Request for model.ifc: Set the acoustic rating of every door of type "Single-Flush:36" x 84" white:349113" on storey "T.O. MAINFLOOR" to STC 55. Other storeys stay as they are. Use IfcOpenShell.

First a look at what the model holds.

```python
import ifcopenshell
import ifcopenshell.util.element

model = ifcopenshell.open("model.ifc")
print(model.schema)
storey = next(s for s in model.by_type("IfcBuildingStorey") if s.Name == "T.O. MAINFLOOR")
doors = [e for e in ifcopenshell.util.element.get_decomposition(storey) if e.is_a("IfcDoor")]
seen = {}
for e in doors:
    element_type = ifcopenshell.util.element.get_type(e)
    key = (element_type.Name if element_type != e and element_type else None, ifcopenshell.util.element.get_pset(e, "Pset_DoorCommon", "AcousticRating"))
    seen[key] = seen.get(key, 0) + 1
for (name, value), count in sorted(seen.items(), key=str):
    print(count, "x", name, "|", value)
```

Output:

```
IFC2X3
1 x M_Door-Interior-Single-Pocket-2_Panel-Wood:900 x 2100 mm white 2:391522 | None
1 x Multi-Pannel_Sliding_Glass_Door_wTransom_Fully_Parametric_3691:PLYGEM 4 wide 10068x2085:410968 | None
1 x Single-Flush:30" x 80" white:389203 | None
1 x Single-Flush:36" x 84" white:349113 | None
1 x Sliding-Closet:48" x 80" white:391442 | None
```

```python
import ifcopenshell
import ifcopenshell.api.pset
import ifcopenshell.util.element

model = ifcopenshell.open("model.ifc")

storey = next(s for s in model.by_type("IfcBuildingStorey") if s.Name == "T.O. MAINFLOOR")
doors = [e for e in ifcopenshell.util.element.get_decomposition(storey) if e.is_a("IfcDoor")]

count = 0
for e in doors:
    element_type = ifcopenshell.util.element.get_type(e)
    if element_type in (None, e) or element_type.Name != 'Single-Flush:36" x 84" white:349113':
        continue
    # add_pset returns the element's existing set when there is one.
    pset = ifcopenshell.api.pset.add_pset(model, product=e, name="Pset_DoorCommon")
    ifcopenshell.api.pset.edit_pset(model, pset=pset, properties={"AcousticRating": "STC 55"})
    count += 1

print(count, "doors updated")

model.write("model_rev.ifc")
```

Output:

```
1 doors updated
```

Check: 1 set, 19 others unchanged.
